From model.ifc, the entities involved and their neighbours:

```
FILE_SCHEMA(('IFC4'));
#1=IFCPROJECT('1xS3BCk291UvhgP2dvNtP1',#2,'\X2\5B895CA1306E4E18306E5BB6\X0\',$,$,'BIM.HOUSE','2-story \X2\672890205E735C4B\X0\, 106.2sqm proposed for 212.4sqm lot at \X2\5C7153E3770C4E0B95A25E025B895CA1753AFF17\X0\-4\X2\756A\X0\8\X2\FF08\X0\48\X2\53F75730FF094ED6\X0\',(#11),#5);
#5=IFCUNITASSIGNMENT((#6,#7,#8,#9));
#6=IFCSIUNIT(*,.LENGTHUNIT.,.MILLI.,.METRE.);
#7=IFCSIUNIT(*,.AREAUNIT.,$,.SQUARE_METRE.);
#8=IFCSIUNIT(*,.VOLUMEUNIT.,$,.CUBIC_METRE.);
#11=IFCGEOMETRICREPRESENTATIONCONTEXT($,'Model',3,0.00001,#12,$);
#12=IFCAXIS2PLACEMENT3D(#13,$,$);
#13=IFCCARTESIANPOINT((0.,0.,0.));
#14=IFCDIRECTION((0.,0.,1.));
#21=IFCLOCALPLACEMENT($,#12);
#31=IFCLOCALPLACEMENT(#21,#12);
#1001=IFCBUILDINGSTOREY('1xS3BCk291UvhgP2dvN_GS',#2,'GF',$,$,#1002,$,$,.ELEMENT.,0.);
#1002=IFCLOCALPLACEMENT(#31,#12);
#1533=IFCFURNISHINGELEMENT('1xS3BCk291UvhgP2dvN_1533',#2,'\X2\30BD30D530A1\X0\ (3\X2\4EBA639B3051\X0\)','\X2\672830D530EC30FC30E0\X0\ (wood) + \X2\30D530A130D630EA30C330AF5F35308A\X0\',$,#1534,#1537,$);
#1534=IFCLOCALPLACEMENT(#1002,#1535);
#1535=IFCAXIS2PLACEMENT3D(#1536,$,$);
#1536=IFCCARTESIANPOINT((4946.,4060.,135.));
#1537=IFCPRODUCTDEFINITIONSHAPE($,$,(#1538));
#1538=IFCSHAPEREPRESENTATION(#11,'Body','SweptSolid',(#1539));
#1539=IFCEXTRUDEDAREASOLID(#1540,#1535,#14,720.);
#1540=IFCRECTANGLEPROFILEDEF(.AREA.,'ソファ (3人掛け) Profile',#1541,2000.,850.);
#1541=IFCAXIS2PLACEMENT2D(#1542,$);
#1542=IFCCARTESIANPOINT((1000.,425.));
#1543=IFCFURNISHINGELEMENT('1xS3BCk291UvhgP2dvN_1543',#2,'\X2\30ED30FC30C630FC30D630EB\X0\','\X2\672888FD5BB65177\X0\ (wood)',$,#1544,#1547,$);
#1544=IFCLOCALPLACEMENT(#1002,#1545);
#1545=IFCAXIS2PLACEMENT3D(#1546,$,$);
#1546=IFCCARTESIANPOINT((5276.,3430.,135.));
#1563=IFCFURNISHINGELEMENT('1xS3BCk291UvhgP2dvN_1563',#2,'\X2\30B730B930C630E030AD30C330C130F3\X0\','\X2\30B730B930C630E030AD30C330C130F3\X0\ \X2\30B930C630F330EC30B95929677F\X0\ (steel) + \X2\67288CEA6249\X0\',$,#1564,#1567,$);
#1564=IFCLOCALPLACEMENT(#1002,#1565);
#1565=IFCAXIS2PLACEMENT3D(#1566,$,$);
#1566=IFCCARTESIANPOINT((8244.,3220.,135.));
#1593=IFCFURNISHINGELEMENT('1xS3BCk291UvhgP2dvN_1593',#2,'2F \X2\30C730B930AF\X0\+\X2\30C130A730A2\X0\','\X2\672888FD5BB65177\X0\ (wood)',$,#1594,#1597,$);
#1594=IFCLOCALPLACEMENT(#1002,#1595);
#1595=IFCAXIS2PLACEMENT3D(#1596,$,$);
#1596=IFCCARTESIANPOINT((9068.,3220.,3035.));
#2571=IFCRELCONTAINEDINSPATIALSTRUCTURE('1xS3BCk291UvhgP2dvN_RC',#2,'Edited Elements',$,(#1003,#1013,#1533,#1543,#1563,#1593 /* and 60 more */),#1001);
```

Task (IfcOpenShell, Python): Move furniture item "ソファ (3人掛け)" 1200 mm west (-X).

```python
import ifcopenshell
import ifcopenshell.api.geometry
import ifcopenshell.util.placement
import ifcopenshell.util.unit

model = ifcopenshell.open("model.ifc")
unit_scale = ifcopenshell.util.unit.calculate_unit_scale(model)

item = model.by_id(1533)
matrix = ifcopenshell.util.placement.get_local_placement(item.ObjectPlacement)
matrix[0, 3] -= 1.2 / unit_scale
ifcopenshell.api.geometry.edit_object_placement(model, product=item, matrix=matrix, is_si=False)

print(ifcopenshell.util.placement.get_local_placement(item.ObjectPlacement).round(3) + 0.0)

model.write("model_rev.ifc")
```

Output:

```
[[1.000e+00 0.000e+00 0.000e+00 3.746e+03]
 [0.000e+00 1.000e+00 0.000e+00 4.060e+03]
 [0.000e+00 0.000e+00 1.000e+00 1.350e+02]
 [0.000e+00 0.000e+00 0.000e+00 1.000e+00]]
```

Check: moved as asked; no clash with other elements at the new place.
